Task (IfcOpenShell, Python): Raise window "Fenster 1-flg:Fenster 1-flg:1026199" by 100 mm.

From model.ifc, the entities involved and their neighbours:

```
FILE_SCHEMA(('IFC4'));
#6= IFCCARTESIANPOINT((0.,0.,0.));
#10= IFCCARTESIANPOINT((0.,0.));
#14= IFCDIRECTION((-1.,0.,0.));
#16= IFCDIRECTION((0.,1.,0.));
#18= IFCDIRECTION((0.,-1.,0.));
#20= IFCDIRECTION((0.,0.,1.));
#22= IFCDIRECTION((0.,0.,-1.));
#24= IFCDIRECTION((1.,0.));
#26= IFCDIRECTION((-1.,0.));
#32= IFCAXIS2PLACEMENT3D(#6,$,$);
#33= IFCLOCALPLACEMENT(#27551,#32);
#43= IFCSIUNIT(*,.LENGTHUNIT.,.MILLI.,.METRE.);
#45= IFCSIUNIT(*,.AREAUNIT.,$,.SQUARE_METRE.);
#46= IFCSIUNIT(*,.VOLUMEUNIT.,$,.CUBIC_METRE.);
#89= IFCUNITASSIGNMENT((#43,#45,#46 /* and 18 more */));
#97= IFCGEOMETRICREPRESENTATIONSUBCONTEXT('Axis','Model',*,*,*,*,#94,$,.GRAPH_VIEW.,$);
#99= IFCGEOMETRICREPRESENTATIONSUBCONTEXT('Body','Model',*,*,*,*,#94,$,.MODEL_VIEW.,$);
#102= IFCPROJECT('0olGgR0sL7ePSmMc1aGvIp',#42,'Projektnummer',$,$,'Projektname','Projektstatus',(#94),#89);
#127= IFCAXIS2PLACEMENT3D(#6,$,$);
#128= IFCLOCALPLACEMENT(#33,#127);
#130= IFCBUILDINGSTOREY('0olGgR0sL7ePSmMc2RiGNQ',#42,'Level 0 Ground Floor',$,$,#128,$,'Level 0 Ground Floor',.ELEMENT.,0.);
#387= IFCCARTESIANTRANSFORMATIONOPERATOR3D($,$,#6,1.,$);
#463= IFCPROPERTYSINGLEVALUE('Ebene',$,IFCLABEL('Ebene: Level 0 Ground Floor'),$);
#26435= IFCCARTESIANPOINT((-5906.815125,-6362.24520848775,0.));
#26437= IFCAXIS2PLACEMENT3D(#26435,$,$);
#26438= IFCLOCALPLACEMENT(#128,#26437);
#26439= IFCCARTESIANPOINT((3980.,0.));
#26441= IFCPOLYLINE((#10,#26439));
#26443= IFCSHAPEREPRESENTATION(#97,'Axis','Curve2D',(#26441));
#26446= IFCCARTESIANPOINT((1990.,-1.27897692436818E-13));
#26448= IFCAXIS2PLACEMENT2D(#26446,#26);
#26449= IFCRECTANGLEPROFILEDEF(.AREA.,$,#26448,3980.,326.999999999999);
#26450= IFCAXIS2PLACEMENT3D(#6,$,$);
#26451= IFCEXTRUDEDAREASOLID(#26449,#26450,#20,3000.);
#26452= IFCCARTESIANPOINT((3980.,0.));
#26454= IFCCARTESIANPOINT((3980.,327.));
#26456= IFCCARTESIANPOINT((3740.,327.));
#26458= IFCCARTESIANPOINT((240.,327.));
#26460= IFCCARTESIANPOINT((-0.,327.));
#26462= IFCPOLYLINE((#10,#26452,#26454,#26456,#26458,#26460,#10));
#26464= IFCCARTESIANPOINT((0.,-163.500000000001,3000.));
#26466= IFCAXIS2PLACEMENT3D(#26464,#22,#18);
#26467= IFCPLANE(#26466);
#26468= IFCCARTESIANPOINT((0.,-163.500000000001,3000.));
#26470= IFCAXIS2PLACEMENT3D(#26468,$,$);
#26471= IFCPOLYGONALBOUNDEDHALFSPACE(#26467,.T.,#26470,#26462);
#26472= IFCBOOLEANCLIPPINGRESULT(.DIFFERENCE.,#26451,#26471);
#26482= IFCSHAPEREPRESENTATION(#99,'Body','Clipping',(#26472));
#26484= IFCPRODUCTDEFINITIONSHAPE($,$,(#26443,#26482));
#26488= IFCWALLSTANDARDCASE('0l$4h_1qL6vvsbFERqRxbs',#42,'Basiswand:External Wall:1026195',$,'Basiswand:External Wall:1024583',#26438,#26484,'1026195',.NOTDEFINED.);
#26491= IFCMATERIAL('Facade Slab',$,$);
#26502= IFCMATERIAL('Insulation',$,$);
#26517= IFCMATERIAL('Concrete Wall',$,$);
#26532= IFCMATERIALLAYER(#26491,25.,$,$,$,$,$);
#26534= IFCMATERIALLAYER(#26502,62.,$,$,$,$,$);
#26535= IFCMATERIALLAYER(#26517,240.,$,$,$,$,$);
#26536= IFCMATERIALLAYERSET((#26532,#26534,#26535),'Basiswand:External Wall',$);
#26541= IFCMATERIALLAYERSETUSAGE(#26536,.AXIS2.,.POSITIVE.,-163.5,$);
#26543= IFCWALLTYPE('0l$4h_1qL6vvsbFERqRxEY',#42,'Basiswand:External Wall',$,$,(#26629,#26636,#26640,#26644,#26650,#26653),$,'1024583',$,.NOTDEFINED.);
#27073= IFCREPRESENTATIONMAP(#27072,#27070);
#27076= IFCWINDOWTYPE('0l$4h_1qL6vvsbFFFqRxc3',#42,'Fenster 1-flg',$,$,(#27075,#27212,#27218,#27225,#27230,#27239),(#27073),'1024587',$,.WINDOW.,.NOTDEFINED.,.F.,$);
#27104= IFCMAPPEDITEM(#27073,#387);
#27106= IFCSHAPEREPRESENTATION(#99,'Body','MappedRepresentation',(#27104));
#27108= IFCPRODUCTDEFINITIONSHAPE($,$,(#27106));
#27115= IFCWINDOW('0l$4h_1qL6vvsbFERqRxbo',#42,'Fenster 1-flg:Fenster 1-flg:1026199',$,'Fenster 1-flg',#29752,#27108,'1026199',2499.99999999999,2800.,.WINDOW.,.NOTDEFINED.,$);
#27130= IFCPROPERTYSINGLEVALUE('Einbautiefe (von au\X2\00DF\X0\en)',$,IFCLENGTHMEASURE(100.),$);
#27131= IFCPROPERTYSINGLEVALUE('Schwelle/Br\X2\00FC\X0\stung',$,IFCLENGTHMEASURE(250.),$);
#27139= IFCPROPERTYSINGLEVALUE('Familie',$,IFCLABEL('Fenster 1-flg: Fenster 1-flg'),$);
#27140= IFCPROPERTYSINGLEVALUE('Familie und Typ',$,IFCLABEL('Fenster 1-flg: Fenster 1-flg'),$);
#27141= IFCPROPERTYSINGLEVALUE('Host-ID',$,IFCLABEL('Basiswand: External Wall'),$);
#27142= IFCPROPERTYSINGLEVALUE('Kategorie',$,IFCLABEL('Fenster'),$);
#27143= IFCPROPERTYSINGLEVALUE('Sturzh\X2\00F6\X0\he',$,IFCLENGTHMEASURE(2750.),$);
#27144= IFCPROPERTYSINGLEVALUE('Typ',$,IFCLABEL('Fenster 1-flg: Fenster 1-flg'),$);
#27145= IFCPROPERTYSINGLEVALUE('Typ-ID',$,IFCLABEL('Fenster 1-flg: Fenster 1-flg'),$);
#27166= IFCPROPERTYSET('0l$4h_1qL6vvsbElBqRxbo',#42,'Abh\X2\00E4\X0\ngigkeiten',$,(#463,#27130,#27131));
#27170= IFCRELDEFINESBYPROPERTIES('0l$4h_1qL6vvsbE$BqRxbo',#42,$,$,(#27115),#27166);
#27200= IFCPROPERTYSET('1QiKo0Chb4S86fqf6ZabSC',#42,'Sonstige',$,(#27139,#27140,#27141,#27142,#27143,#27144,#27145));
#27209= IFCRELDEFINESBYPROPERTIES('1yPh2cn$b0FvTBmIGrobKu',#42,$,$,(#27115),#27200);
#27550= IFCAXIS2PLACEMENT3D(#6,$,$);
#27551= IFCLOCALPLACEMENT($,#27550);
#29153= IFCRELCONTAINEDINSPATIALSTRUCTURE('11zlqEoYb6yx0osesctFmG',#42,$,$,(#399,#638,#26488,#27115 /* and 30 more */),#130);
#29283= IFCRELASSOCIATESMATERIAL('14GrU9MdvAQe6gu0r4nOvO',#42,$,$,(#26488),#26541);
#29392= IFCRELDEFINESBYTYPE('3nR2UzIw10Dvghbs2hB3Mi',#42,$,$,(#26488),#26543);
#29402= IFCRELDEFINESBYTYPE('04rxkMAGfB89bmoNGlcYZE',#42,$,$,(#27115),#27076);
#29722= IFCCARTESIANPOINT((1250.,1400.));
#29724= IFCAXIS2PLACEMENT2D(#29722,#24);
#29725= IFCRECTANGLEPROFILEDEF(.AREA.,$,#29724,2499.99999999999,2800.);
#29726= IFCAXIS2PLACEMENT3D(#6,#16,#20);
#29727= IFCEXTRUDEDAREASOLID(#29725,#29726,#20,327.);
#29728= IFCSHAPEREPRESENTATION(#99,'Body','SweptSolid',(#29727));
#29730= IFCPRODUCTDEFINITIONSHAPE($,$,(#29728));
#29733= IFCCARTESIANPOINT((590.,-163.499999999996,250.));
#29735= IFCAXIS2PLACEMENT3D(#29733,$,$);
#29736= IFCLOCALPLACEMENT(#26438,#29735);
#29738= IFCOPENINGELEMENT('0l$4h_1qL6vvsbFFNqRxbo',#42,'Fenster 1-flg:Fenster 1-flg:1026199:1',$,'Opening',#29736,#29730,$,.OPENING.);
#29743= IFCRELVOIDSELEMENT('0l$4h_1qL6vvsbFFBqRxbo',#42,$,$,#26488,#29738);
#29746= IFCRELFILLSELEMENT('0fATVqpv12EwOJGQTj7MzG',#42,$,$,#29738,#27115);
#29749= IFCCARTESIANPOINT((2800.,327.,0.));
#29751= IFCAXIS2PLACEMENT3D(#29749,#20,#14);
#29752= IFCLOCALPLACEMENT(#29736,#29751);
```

```python
import numpy as np
import ifcopenshell
import ifcopenshell.api.geometry
import ifcopenshell.api.pset
import ifcopenshell.util.element
import ifcopenshell.util.placement
import ifcopenshell.util.unit

model = ifcopenshell.open("model.ifc")
unit_scale = ifcopenshell.util.unit.calculate_unit_scale(model)

window = model.by_guid("0l$4h_1qL6vvsbFERqRxbo")
opening = window.FillsVoids[0].RelatingOpeningElement
dz = 0.1 / unit_scale

shift = np.array([0.0, 0.0, dz])
# The window is placed relative to its opening, so it follows when the opening moves.
matrix = ifcopenshell.util.placement.get_local_placement(opening.ObjectPlacement)
matrix[:3, 3] += shift
ifcopenshell.api.geometry.edit_object_placement(
    model, product=opening, matrix=matrix, is_si=False, should_transform_children=True
)

# Keep the stored heights in step.
pset = model.by_id(ifcopenshell.util.element.get_pset(window, "Abhängigkeiten", should_inherit=False)["id"])
ifcopenshell.api.pset.edit_pset(model, pset=pset, properties={
    "Schwelle/Brüstung": model.create_entity("IfcLengthMeasure", ifcopenshell.util.element.get_pset(window, "Abhängigkeiten", "Schwelle/Brüstung") + dz),
})
pset = model.by_id(ifcopenshell.util.element.get_pset(window, "Sonstige", should_inherit=False)["id"])
ifcopenshell.api.pset.edit_pset(model, pset=pset, properties={
    "Sturzhöhe": model.create_entity("IfcLengthMeasure", ifcopenshell.util.element.get_pset(window, "Sonstige", "Sturzhöhe") + dz),
})

print(f"moved by {dz * unit_scale:+.3f} m")

model.write("model_rev.ifc")
```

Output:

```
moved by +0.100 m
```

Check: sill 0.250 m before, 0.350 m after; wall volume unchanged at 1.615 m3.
